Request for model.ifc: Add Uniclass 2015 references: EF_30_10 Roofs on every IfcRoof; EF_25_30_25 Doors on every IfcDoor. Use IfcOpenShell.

First a look at what the model holds.

```python
import ifcopenshell

model = ifcopenshell.open("model.ifc")
print(model.schema)
print("classifications:", [c.Name for c in model.by_type("IfcClassification")])
for ifc_class in ("IfcDoor", "IfcRoof", "IfcStair", "IfcWall", "IfcWindow"):
    print(ifc_class, len(model.by_type(ifc_class)))
```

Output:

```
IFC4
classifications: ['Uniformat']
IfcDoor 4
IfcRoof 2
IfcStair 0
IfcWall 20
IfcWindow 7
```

```python
import ifcopenshell
import ifcopenshell.api.classification

model = ifcopenshell.open("model.ifc")

system = ifcopenshell.api.classification.add_classification(model, classification="Uniclass 2015")

codes = {
    "IfcRoof": ("EF_30_10", "Roofs"),
    "IfcDoor": ("EF_25_30_25", "Doors"),
}
for ifc_class, (code, name) in codes.items():
    products = model.by_type(ifc_class)
    ifcopenshell.api.classification.add_reference(
        model, products=products, classification=system, identification=code, name=name
    )
    print(code, len(products))

model.write("model_v2.ifc")
```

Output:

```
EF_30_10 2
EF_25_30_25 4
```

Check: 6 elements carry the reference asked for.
